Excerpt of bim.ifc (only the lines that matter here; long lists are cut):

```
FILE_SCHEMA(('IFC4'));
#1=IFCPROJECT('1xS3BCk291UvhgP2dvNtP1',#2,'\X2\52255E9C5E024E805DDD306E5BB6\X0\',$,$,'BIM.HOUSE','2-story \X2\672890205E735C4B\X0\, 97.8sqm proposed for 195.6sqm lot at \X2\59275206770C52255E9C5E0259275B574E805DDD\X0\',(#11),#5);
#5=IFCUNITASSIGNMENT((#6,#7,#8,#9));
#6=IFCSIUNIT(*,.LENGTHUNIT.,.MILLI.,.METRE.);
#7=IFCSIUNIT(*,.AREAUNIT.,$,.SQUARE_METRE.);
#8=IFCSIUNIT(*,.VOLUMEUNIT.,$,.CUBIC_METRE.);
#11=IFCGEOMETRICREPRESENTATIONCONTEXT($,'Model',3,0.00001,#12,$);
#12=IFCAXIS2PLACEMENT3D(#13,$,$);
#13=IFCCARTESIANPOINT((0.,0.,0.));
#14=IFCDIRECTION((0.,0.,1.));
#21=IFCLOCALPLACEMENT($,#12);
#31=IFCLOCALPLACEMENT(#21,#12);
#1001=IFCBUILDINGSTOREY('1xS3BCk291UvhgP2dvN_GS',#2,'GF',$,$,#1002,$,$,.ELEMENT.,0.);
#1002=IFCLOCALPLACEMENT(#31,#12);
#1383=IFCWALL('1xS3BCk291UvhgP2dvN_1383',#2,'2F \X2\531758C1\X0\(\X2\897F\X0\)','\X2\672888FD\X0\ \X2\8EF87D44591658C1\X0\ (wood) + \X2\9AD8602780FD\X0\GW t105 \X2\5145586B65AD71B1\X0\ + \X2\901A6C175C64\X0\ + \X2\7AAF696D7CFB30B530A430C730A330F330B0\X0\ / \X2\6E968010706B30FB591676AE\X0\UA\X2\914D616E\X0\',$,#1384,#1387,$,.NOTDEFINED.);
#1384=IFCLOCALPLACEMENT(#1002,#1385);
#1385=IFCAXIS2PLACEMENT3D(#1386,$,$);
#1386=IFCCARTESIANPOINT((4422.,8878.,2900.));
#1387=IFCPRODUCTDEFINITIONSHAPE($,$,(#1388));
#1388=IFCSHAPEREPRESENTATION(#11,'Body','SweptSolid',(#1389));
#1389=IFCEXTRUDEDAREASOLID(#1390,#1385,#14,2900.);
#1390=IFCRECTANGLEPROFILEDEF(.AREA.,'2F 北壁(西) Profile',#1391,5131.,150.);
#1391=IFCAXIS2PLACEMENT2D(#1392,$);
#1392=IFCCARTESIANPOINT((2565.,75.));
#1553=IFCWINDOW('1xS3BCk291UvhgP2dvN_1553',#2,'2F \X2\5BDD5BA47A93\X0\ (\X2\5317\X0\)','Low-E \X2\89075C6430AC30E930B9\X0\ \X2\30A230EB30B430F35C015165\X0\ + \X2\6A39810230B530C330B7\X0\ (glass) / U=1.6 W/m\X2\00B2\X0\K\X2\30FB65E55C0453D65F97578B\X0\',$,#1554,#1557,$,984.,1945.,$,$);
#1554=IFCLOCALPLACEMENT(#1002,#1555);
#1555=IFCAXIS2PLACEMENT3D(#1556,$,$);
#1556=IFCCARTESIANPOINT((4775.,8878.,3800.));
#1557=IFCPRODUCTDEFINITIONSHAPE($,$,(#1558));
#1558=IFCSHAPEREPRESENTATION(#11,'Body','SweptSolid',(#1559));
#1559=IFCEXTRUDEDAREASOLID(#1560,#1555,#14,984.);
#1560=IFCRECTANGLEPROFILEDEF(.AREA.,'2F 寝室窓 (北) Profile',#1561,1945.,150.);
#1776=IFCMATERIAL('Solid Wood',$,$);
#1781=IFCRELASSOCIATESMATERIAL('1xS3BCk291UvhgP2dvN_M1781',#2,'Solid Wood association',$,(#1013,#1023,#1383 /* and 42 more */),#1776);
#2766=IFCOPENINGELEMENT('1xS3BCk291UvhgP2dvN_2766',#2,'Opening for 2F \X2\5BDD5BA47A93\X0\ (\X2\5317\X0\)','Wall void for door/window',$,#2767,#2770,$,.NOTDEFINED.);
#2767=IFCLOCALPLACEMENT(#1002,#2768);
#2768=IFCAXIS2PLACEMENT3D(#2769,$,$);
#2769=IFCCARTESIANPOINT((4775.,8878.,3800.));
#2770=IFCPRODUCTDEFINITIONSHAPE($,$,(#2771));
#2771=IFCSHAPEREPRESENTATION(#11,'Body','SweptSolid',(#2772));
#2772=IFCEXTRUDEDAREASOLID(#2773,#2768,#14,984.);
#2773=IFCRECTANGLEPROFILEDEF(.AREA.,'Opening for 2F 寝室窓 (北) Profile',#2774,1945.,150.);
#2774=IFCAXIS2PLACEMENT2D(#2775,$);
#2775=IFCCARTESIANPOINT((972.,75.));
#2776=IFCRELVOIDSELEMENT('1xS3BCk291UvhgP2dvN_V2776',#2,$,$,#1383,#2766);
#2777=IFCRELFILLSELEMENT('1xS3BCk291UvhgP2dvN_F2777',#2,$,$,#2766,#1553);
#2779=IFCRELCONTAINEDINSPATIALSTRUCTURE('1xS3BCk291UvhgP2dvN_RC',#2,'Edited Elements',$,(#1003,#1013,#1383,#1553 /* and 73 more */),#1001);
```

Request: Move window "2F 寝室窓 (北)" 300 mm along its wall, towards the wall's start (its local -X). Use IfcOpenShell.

```python
import ifcopenshell
import ifcopenshell.api.geometry
import ifcopenshell.util.placement

model = ifcopenshell.open("bim.ifc")

window = model.by_guid("1xS3BCk291UvhgP2dvN_1553")
opening = window.FillsVoids[0].RelatingOpeningElement
wall = opening.VoidsElements[0].RelatingBuildingElement

wall_matrix = ifcopenshell.util.placement.get_local_placement(wall.ObjectPlacement)
shift = wall_matrix[:3, 0] * -300.0
before = ifcopenshell.util.placement.get_local_placement(window.ObjectPlacement)[:3, 3].copy()

# The window is not placed relative to its opening, so move both.
for product in (opening, window):
    matrix = ifcopenshell.util.placement.get_local_placement(product.ObjectPlacement)
    matrix[:3, 3] += shift
    ifcopenshell.api.geometry.edit_object_placement(model, product=product, matrix=matrix, is_si=False)

after = ifcopenshell.util.placement.get_local_placement(window.ObjectPlacement)[:3, 3]
print("window moved by", (after - before).round(3) + 0.0)

model.write("bim_rev.ifc")
```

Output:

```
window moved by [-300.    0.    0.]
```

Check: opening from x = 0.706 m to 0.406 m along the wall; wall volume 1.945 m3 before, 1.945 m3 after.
